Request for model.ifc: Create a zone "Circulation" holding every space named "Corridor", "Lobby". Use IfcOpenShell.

First a look at what the model holds.

```python
import ifcopenshell

model = ifcopenshell.open("model.ifc")
print(model.schema)
seen = {}
for space in model.by_type("IfcSpace"):
    seen[space.LongName] = seen.get(space.LongName, 0) + 1
for name, count in sorted(seen.items(), key=str):
    print(count, "x", name)
print("zones:", [z.Name for z in model.by_type("IfcZone")][:20])
```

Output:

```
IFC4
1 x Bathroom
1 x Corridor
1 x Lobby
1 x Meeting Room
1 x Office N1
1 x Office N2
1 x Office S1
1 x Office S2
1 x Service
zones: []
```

```python
import ifcopenshell
import ifcopenshell.api.group
import ifcopenshell.api.root

model = ifcopenshell.open("model.ifc")

names = {"Corridor", "Lobby"}
spaces = [s for s in model.by_type("IfcSpace") if s.LongName in names]

zone = ifcopenshell.api.root.create_entity(model, ifc_class="IfcZone", name="Circulation")
ifcopenshell.api.group.assign_group(model, products=spaces, group=zone)
print(len(spaces), "spaces in", zone.Name)

model.write("model_edited.ifc")
```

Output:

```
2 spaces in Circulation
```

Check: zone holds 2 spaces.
